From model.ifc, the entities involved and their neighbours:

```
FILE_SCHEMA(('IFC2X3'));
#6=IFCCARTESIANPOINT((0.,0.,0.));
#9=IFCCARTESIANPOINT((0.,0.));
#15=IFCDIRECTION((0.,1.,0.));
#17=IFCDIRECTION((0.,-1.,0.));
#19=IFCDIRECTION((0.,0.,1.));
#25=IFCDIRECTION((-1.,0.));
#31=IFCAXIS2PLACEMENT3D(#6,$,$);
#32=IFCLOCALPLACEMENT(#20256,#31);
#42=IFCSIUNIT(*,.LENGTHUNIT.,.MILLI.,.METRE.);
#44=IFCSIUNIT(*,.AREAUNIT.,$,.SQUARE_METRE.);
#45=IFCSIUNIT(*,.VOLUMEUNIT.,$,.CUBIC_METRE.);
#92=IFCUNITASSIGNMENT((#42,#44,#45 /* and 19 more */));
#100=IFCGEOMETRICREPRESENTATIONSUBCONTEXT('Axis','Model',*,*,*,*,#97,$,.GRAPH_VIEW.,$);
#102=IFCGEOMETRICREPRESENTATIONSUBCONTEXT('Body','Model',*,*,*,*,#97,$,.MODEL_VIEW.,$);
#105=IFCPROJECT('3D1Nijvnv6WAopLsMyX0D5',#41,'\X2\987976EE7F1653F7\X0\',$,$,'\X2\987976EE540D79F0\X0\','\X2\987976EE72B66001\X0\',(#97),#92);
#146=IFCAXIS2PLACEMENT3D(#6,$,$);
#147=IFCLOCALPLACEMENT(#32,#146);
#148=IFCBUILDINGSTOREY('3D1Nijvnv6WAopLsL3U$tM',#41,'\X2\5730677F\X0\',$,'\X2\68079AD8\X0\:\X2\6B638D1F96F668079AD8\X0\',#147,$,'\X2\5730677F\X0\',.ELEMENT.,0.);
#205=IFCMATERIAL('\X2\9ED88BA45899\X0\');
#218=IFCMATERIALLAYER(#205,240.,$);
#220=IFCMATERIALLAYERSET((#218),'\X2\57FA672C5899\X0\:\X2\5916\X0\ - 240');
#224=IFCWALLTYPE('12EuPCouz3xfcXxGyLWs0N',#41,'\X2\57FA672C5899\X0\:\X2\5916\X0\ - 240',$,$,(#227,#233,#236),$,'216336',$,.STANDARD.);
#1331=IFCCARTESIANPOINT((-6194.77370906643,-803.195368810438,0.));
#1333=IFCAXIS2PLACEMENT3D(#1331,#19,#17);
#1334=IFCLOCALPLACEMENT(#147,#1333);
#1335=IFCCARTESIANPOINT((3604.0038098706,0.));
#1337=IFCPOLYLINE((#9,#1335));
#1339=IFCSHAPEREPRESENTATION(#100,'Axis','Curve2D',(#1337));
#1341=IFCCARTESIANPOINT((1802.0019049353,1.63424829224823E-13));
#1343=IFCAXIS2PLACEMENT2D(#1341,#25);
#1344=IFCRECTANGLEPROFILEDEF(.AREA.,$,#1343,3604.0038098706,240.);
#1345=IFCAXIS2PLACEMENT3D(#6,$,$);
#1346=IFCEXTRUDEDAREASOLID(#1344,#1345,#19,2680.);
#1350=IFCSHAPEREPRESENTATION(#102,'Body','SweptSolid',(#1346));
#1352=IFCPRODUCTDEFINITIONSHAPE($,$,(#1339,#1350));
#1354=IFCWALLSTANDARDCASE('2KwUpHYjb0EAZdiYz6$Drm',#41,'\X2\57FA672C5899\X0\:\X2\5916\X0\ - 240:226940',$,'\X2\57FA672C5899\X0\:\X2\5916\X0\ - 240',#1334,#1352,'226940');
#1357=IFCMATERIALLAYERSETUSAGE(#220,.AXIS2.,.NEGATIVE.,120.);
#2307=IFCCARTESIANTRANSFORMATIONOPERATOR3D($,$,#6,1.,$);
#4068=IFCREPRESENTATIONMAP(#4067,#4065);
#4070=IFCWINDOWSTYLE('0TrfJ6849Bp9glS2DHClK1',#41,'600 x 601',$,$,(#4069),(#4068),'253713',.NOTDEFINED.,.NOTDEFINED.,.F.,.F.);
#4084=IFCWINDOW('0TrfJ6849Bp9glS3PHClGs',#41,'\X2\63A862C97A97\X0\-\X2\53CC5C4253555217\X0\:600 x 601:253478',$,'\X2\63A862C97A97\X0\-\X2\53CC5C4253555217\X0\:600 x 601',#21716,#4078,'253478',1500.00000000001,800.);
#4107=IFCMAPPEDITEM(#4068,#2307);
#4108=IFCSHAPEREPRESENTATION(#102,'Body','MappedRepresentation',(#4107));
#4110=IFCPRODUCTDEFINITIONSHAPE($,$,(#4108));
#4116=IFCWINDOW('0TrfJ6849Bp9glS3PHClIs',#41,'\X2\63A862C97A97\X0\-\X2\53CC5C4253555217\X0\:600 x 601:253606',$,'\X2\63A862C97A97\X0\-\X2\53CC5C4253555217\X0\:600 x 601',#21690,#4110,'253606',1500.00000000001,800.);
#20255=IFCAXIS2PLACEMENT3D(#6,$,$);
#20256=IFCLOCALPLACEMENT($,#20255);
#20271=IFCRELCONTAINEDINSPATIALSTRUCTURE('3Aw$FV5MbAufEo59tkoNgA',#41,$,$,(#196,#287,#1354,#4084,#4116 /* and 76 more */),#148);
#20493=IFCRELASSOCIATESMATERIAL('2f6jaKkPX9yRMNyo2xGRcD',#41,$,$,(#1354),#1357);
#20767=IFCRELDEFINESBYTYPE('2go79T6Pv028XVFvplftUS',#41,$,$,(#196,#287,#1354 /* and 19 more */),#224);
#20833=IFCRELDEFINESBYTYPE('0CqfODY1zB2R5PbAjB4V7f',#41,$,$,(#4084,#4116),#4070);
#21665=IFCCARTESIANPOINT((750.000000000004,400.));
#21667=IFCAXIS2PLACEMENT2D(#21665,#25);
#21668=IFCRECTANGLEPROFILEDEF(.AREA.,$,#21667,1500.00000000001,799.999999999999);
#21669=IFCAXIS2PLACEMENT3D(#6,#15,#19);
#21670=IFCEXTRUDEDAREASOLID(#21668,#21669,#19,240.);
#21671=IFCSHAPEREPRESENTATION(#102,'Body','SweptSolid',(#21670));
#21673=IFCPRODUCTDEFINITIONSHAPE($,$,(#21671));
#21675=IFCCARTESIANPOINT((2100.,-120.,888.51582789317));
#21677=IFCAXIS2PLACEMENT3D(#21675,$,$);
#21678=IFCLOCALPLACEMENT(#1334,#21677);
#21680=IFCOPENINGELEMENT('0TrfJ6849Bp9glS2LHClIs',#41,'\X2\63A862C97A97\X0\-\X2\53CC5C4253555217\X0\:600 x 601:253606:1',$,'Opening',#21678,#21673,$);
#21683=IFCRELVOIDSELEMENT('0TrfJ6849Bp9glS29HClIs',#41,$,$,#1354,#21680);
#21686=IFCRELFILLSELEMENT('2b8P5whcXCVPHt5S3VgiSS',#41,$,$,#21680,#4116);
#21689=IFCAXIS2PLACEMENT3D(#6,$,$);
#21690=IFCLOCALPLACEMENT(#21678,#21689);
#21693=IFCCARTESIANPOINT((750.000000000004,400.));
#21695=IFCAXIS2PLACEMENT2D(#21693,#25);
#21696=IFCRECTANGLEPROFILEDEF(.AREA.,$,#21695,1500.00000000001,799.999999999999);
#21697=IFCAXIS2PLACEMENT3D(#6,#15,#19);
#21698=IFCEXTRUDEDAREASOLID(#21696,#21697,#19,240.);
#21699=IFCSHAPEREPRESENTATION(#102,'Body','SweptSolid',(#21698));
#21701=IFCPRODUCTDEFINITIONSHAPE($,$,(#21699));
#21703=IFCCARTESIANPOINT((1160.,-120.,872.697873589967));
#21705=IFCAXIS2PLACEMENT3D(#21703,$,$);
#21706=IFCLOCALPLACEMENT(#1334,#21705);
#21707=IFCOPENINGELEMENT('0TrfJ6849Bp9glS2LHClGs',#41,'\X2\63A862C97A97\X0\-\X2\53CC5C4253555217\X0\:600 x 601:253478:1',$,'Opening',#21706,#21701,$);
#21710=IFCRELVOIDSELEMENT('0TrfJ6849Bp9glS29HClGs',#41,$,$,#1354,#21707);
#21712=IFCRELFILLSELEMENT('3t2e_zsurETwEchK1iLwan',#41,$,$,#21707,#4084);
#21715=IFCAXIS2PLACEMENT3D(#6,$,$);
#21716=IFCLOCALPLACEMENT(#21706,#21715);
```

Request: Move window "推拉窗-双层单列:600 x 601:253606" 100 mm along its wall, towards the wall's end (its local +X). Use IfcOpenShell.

```python
import ifcopenshell
import ifcopenshell.api.geometry
import ifcopenshell.util.placement

model = ifcopenshell.open("model.ifc")

window = model.by_guid("0TrfJ6849Bp9glS3PHClIs")
opening = window.FillsVoids[0].RelatingOpeningElement
wall = opening.VoidsElements[0].RelatingBuildingElement

wall_matrix = ifcopenshell.util.placement.get_local_placement(wall.ObjectPlacement)
shift = wall_matrix[:3, 0] * 100.0
before = ifcopenshell.util.placement.get_local_placement(window.ObjectPlacement)[:3, 3].copy()

# The window is placed relative to its opening, so it follows when the opening moves.
matrix = ifcopenshell.util.placement.get_local_placement(opening.ObjectPlacement)
matrix[:3, 3] += shift
ifcopenshell.api.geometry.edit_object_placement(
    model, product=opening, matrix=matrix, is_si=False, should_transform_children=True
)

after = ifcopenshell.util.placement.get_local_placement(window.ObjectPlacement)[:3, 3]
print("window moved by", (after - before).round(3) + 0.0)

model.write("model_edited.ifc")
```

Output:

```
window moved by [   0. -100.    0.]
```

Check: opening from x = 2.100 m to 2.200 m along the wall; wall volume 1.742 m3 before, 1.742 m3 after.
